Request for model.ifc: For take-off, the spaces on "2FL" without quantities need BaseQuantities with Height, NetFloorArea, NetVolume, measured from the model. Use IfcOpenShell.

First a look at what the model holds.

```python
import ifcopenshell
import ifcopenshell.util.element
import ifcopenshell.util.unit

model = ifcopenshell.open("model.ifc")
print(model.schema)
for unit_type in ("LENGTHUNIT", "AREAUNIT", "VOLUMEUNIT"):
    print(unit_type, ifcopenshell.util.unit.calculate_unit_scale(model, unit_type))
storey = next(s for s in model.by_type("IfcBuildingStorey") if s.Name == "2FL")
spaces = [e for e in ifcopenshell.util.element.get_decomposition(storey) if e.is_a("IfcSpace")]
for e in sorted(spaces, key=lambda e: e.id()):
    print(e.id(), e.is_a(), e.Name, list(ifcopenshell.util.element.get_psets(e, qtos_only=True)), sep=" | ")
```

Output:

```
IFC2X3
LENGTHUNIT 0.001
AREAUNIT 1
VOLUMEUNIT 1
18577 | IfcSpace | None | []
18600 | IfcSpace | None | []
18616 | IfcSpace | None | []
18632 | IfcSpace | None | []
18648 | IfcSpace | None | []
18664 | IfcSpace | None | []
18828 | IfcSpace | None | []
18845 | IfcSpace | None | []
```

```python
import ifcopenshell
import ifcopenshell.api.pset
import ifcopenshell.geom
import ifcopenshell.util.element
import ifcopenshell.util.shape
import ifcopenshell.util.unit

model = ifcopenshell.open("model.ifc")
unit_scale = ifcopenshell.util.unit.calculate_unit_scale(model)
area_scale = ifcopenshell.util.unit.calculate_unit_scale(model, "AREAUNIT")
volume_scale = ifcopenshell.util.unit.calculate_unit_scale(model, "VOLUMEUNIT")
settings = ifcopenshell.geom.settings()

storey = next(s for s in model.by_type("IfcBuildingStorey") if s.Name == "2FL")
spaces = [e for e in ifcopenshell.util.element.get_decomposition(storey) if e.is_a("IfcSpace")]

for e in sorted(spaces, key=lambda e: e.id()):
    if ifcopenshell.util.element.get_psets(e, qtos_only=True, should_inherit=False):
        continue
    # Geometry comes back in metres, in the element's own axes.
    shape = ifcopenshell.geom.create_shape(settings, e)
    values = {
        "Height": ifcopenshell.util.shape.get_z(shape.geometry) / unit_scale,
        "NetFloorArea": ifcopenshell.util.shape.get_footprint_area(shape.geometry) / area_scale,
        "NetVolume": ifcopenshell.util.shape.get_volume(shape.geometry) / volume_scale,
    }
    qto = ifcopenshell.api.pset.add_qto(model, product=e, name="BaseQuantities")
    ifcopenshell.api.pset.edit_qto(model, qto=qto, properties=values)
    print(e.id(), {k: round(v, 3) for k, v in values.items()})

model.write("model_updated.ifc")
```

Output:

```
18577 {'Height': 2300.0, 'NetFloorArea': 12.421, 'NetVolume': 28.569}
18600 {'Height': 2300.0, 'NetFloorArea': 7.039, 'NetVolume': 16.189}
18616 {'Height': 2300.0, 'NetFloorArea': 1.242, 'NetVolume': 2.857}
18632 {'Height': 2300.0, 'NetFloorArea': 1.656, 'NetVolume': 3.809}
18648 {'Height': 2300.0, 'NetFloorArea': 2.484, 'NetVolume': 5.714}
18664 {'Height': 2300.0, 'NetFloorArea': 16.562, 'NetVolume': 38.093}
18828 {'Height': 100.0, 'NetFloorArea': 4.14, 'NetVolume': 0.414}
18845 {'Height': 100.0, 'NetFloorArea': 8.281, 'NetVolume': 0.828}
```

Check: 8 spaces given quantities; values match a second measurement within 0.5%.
